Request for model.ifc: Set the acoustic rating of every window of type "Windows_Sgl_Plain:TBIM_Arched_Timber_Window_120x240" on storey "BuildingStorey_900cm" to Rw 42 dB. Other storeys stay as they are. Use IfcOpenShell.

First a look at what the model holds.

```python
import ifcopenshell
import ifcopenshell.util.element

model = ifcopenshell.open("model.ifc")
print(model.schema)
storey = next(s for s in model.by_type("IfcBuildingStorey") if s.Name == "BuildingStorey_900cm")
windows = [e for e in ifcopenshell.util.element.get_decomposition(storey) if e.is_a("IfcWindow")]
seen = {}
for e in windows:
    element_type = ifcopenshell.util.element.get_type(e)
    key = (element_type.Name if element_type != e and element_type else None, ifcopenshell.util.element.get_pset(e, "Pset_WindowCommon", "AcousticRating"))
    seen[key] = seen.get(key, 0) + 1
for (name, value), count in sorted(seen.items(), key=str):
    print(count, "x", name, "|", value)
```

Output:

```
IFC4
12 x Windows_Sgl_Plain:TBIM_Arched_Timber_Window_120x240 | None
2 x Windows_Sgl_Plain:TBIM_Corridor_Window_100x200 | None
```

```python
import ifcopenshell
import ifcopenshell.api.pset
import ifcopenshell.util.element

model = ifcopenshell.open("model.ifc")

storey = next(s for s in model.by_type("IfcBuildingStorey") if s.Name == "BuildingStorey_900cm")
windows = [e for e in ifcopenshell.util.element.get_decomposition(storey) if e.is_a("IfcWindow")]

count = 0
for e in windows:
    element_type = ifcopenshell.util.element.get_type(e)
    if element_type in (None, e) or element_type.Name != "Windows_Sgl_Plain:TBIM_Arched_Timber_Window_120x240":
        continue
    # add_pset returns the element's existing set when there is one.
    pset = ifcopenshell.api.pset.add_pset(model, product=e, name="Pset_WindowCommon")
    ifcopenshell.api.pset.edit_pset(model, pset=pset, properties={"AcousticRating": "Rw 42 dB"})
    count += 1

print(count, "windows updated")

model.write("model_updated.ifc")
```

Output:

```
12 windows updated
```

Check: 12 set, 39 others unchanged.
